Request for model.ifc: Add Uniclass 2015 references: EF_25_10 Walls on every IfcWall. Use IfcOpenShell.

First a look at what the model holds.

```python
import ifcopenshell

model = ifcopenshell.open("model.ifc")
print(model.schema)
print("classifications:", [c.Name for c in model.by_type("IfcClassification")])
for ifc_class in ("IfcDoor", "IfcRoof", "IfcStair", "IfcWall", "IfcWindow"):
    print(ifc_class, len(model.by_type(ifc_class)))
```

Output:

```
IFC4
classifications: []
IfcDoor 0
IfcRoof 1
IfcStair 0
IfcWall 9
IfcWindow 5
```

```python
import ifcopenshell
import ifcopenshell.api.classification

model = ifcopenshell.open("model.ifc")

system = ifcopenshell.api.classification.add_classification(model, classification="Uniclass 2015")

codes = {
    "IfcWall": ("EF_25_10", "Walls"),
}
for ifc_class, (code, name) in codes.items():
    products = model.by_type(ifc_class)
    ifcopenshell.api.classification.add_reference(
        model, products=products, classification=system, identification=code, name=name
    )
    print(code, len(products))

model.write("model-out.ifc")
```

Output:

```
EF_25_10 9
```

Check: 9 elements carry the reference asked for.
